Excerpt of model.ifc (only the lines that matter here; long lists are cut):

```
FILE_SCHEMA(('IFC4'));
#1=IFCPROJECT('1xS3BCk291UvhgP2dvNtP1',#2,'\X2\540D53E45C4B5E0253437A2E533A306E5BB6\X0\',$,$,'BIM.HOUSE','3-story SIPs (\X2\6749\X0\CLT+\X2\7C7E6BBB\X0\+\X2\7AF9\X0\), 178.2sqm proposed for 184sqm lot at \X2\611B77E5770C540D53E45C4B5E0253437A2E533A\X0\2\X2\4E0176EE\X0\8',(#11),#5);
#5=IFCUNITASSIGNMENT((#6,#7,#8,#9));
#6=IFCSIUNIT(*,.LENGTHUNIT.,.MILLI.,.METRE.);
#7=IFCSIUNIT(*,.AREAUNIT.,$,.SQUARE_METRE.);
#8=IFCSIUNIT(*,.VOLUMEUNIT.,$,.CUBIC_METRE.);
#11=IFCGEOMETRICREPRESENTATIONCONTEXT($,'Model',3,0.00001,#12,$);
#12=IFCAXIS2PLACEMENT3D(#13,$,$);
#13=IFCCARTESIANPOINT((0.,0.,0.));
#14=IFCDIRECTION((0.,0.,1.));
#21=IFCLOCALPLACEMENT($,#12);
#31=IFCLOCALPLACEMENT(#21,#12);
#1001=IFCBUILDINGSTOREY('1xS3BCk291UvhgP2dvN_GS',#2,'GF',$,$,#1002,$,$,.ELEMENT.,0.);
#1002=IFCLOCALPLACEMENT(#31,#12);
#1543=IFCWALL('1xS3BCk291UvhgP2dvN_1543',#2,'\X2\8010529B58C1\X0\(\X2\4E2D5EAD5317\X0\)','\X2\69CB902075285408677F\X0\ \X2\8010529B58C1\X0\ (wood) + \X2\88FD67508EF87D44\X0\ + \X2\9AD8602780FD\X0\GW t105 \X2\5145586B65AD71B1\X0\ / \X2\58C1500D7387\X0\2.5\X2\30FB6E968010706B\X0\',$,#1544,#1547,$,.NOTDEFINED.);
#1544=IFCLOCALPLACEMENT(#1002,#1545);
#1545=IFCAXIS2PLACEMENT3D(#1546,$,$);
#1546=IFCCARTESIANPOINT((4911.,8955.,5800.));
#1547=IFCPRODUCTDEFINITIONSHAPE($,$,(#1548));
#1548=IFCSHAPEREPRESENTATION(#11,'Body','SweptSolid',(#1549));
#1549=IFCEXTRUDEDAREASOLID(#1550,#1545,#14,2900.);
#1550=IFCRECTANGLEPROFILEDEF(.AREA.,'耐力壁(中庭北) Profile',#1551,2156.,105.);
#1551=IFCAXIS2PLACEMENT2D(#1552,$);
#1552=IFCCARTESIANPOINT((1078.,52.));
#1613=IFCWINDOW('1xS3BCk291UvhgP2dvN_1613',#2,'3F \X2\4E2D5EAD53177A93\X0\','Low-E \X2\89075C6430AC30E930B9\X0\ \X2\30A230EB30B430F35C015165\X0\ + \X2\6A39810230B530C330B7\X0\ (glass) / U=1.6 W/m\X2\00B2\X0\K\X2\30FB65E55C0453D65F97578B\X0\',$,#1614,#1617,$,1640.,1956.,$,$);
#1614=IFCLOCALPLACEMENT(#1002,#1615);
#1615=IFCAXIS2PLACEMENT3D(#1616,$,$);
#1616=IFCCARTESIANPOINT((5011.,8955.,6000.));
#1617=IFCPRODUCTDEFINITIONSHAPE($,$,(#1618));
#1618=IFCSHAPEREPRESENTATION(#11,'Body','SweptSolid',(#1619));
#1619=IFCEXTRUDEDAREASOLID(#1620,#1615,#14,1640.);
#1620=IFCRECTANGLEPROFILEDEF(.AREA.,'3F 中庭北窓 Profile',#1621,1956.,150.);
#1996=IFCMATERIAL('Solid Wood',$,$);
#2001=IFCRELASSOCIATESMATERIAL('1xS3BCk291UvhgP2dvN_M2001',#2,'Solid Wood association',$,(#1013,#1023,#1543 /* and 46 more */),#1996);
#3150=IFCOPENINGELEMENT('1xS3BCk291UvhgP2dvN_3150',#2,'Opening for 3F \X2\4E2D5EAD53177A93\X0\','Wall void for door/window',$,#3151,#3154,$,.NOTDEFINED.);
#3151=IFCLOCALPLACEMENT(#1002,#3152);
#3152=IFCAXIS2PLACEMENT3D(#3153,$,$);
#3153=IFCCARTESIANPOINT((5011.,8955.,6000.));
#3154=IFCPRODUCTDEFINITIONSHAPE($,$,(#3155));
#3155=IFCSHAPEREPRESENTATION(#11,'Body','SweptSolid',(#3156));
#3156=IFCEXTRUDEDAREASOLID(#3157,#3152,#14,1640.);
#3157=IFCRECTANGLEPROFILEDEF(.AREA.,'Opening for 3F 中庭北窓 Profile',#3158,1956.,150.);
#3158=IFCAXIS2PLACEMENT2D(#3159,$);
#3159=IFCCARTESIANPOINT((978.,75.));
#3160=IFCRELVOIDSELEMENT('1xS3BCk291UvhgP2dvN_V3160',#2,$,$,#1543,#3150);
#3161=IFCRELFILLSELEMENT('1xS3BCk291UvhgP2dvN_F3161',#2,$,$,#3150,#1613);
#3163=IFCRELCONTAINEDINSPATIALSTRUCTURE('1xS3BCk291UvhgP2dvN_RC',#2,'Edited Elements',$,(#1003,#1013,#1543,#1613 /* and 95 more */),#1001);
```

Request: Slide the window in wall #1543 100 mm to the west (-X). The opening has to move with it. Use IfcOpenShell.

```python
import ifcopenshell
import ifcopenshell.api.geometry
import ifcopenshell.util.placement

model = ifcopenshell.open("model.ifc")

window = model.by_guid("1xS3BCk291UvhgP2dvN_1613")
opening = window.FillsVoids[0].RelatingOpeningElement
wall = opening.VoidsElements[0].RelatingBuildingElement

wall_matrix = ifcopenshell.util.placement.get_local_placement(wall.ObjectPlacement)
shift = wall_matrix[:3, 0] * -100.0
before = ifcopenshell.util.placement.get_local_placement(window.ObjectPlacement)[:3, 3].copy()

# The window is not placed relative to its opening, so move both.
for product in (opening, window):
    matrix = ifcopenshell.util.placement.get_local_placement(product.ObjectPlacement)
    matrix[:3, 3] += shift
    ifcopenshell.api.geometry.edit_object_placement(model, product=product, matrix=matrix, is_si=False)

after = ifcopenshell.util.placement.get_local_placement(window.ObjectPlacement)[:3, 3]
print("window moved by", (after - before).round(3) + 0.0)

model.write("model-out.ifc")
```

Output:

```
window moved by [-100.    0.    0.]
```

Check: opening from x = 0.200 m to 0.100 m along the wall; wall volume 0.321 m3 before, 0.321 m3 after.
